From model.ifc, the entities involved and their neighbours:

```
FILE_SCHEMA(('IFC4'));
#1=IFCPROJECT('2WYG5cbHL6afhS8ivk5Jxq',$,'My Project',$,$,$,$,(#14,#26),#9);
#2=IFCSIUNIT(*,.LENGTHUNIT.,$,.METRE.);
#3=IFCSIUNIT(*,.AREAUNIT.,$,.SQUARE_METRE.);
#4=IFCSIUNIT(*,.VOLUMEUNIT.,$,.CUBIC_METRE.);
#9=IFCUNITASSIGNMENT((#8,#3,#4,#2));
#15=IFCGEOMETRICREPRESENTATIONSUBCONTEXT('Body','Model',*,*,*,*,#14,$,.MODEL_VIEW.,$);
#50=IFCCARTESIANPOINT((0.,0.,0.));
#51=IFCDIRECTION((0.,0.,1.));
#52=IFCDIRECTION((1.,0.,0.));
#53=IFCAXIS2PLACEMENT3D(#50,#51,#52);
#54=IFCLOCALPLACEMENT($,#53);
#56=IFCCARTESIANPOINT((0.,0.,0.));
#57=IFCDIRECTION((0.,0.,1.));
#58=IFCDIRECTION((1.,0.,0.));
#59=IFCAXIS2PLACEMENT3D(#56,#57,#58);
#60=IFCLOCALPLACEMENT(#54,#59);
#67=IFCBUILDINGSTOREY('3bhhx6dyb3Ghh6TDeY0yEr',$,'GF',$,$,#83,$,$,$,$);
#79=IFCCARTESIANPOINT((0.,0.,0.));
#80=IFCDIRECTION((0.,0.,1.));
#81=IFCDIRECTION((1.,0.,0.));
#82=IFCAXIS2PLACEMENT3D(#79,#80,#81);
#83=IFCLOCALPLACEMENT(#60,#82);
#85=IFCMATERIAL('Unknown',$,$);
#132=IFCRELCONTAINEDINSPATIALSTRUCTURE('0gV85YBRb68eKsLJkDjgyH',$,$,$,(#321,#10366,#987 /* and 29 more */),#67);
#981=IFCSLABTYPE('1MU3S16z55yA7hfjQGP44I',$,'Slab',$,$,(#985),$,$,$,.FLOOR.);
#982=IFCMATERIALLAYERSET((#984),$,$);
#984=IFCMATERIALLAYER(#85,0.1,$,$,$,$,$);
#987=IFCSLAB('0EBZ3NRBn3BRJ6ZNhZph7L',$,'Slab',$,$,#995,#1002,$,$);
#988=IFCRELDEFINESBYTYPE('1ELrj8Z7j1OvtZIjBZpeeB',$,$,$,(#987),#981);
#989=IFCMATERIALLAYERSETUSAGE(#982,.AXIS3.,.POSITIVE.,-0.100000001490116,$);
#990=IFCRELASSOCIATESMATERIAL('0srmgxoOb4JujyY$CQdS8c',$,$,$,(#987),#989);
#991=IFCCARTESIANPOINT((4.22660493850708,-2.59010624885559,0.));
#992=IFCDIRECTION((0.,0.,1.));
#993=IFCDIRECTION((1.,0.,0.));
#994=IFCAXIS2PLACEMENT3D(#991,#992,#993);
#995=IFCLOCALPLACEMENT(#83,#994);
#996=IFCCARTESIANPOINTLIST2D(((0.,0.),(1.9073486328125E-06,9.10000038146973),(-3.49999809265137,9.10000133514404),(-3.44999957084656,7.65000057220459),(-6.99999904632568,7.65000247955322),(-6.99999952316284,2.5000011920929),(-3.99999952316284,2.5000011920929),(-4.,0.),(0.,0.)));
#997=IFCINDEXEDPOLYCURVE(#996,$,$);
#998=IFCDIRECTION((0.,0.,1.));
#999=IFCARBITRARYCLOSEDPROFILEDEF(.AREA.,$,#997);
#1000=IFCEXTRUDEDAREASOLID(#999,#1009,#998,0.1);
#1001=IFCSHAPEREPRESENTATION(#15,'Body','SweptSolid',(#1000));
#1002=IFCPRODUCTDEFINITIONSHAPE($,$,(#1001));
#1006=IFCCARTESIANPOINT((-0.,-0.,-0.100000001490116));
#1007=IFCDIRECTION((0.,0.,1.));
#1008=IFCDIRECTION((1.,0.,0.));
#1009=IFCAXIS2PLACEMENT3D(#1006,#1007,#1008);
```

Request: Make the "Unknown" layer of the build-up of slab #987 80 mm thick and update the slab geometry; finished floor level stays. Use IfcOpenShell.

```python
import ifcopenshell
import ifcopenshell.util.element
import ifcopenshell.util.representation

model = ifcopenshell.open("model.ifc")

layer_set = model.by_id(982)
layer = next(l for l in layer_set.MaterialLayers if l.Material and l.Material.Name == "Unknown")
change = 0.08 - layer.LayerThickness
layer.LayerThickness += change

# Geometry does not follow the layer set by itself.
slabs = [e for e in ifcopenshell.util.element.get_elements_by_material(model, layer_set) if e.is_a("IfcSlab")]
for slab in sorted(slabs, key=lambda e: e.id()):
    body = ifcopenshell.util.representation.get_representation(slab, "Model", "Body")
    solid = body.Items[0]
    old_depth = solid.Depth
    solid.Depth += change
    # Extruded upwards: lower the start of the extrusion so the top stays.
    x, y, z = solid.Position.Location.Coordinates
    solid.Position.Location = model.createIfcCartesianPoint((x, y, z - change))
    print(slab.id(), f"{old_depth:g} -> {solid.Depth:g}")

# The layers are counted up from the underside, which has moved.
for usage in {ifcopenshell.util.element.get_material(slab) for slab in slabs}:
    usage.OffsetFromReferenceLine -= change

model.write("model_updated.ifc")
```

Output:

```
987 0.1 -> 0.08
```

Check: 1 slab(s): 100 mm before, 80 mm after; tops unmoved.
